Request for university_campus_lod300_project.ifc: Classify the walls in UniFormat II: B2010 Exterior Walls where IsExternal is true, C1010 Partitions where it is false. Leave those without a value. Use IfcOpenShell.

First a look at what the model holds.

```python
import ifcopenshell
import ifcopenshell.util.element

model = ifcopenshell.open("university_campus_lod300_project.ifc")
print(model.schema)
print("classifications:", [c.Name for c in model.by_type("IfcClassification")])
values = [ifcopenshell.util.element.get_pset(e, "Pset_WallCommon", "IsExternal") for e in model.by_type("IfcWall")]
for value in (True, False, None):
    print("IsExternal", value, values.count(value))
```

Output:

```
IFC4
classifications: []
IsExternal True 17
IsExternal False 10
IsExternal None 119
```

```python
import ifcopenshell
import ifcopenshell.api.classification
import ifcopenshell.util.element

model = ifcopenshell.open("university_campus_lod300_project.ifc")

system = ifcopenshell.api.classification.add_classification(model, classification="UniFormat II")

walls = model.by_type("IfcWall")
external = {e: ifcopenshell.util.element.get_pset(e, "Pset_WallCommon", "IsExternal") for e in walls}
for flag, code, name in ((True, "B2010", "Exterior Walls"), (False, "C1010", "Partitions")):
    products = [e for e in walls if external[e] is flag]
    ifcopenshell.api.classification.add_reference(
        model, products=products, classification=system, identification=code, name=name
    )
    print(code, len(products))

model.write("university_campus_lod300_project_rev.ifc")
```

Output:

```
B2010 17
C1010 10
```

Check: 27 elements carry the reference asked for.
